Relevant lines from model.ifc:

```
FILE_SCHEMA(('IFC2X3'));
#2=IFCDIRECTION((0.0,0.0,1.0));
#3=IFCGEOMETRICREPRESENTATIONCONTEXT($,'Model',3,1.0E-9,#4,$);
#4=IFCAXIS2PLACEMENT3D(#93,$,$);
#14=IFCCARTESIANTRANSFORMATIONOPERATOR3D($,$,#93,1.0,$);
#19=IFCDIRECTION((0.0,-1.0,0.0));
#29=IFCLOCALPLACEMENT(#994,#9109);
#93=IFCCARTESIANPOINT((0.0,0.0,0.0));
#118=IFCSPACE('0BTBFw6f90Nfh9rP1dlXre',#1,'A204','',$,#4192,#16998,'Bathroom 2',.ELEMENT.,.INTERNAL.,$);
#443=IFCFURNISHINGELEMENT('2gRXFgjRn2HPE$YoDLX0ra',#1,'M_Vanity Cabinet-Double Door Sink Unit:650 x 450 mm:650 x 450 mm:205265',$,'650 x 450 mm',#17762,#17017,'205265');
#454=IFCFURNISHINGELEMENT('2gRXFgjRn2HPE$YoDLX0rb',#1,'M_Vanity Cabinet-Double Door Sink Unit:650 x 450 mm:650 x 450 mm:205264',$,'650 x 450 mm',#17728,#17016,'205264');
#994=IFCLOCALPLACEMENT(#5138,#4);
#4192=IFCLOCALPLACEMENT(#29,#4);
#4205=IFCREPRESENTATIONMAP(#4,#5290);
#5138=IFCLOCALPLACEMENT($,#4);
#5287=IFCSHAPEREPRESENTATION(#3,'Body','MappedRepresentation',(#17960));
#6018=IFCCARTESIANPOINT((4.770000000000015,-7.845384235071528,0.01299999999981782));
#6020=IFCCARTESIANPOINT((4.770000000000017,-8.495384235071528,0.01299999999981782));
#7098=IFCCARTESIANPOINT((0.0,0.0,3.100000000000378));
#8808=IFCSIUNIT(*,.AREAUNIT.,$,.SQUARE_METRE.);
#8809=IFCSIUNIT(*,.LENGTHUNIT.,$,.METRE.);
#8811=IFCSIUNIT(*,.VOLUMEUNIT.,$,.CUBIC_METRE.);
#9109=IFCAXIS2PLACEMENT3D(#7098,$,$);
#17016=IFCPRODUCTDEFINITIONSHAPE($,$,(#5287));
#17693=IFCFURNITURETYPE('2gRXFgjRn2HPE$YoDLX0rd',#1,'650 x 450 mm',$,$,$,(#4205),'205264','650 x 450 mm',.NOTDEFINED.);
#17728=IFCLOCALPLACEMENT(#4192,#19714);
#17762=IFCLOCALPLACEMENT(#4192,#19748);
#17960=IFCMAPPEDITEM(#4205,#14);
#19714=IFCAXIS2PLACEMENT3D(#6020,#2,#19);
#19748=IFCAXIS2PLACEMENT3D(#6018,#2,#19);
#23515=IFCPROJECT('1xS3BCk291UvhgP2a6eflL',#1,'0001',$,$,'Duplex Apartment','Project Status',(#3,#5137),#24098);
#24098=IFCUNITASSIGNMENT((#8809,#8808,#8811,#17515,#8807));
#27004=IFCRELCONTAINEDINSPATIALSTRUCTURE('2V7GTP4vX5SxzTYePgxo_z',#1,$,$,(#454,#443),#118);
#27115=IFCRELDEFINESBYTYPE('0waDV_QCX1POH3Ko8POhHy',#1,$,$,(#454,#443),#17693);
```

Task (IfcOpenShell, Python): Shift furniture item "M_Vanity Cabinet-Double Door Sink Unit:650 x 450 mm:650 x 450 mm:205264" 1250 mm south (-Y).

```python
import ifcopenshell
import ifcopenshell.api.geometry
import ifcopenshell.util.placement
import ifcopenshell.util.unit

model = ifcopenshell.open("model.ifc")
unit_scale = ifcopenshell.util.unit.calculate_unit_scale(model)

item = model.by_guid("2gRXFgjRn2HPE$YoDLX0rb")
matrix = ifcopenshell.util.placement.get_local_placement(item.ObjectPlacement)
matrix[1, 3] -= 1.25 / unit_scale
ifcopenshell.api.geometry.edit_object_placement(model, product=item, matrix=matrix, is_si=False)

print(ifcopenshell.util.placement.get_local_placement(item.ObjectPlacement).round(3) + 0.0)

model.write("model_rev.ifc")
```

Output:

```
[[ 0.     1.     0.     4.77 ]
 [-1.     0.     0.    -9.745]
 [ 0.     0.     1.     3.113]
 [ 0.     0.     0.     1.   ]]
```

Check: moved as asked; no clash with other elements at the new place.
